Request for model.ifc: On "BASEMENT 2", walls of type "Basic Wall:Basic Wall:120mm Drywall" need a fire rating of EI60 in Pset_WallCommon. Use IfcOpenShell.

First a look at what the model holds.

```python
import ifcopenshell
import ifcopenshell.util.element

model = ifcopenshell.open("model.ifc")
print(model.schema)
storey = next(s for s in model.by_type("IfcBuildingStorey") if s.Name == "BASEMENT 2")
walls = [e for e in ifcopenshell.util.element.get_decomposition(storey) if e.is_a("IfcWall")]
seen = {}
for e in walls:
    element_type = ifcopenshell.util.element.get_type(e)
    key = (element_type.Name if element_type != e and element_type else None, ifcopenshell.util.element.get_pset(e, "Pset_WallCommon", "FireRating"))
    seen[key] = seen.get(key, 0) + 1
for (name, value), count in sorted(seen.items(), key=str):
    print(count, "x", name, "|", value)
```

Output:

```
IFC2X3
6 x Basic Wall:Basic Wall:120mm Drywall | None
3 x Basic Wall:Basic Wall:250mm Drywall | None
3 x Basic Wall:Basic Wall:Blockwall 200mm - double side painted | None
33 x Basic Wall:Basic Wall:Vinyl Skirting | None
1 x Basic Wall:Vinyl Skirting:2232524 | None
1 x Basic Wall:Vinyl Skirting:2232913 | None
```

```python
import ifcopenshell
import ifcopenshell.api.pset
import ifcopenshell.util.element

model = ifcopenshell.open("model.ifc")

storey = next(s for s in model.by_type("IfcBuildingStorey") if s.Name == "BASEMENT 2")
walls = [e for e in ifcopenshell.util.element.get_decomposition(storey) if e.is_a("IfcWall")]

count = 0
for e in walls:
    element_type = ifcopenshell.util.element.get_type(e)
    if element_type in (None, e) or element_type.Name != "Basic Wall:Basic Wall:120mm Drywall":
        continue
    # add_pset returns the element's existing set when there is one.
    pset = ifcopenshell.api.pset.add_pset(model, product=e, name="Pset_WallCommon")
    ifcopenshell.api.pset.edit_pset(model, pset=pset, properties={"FireRating": "EI60"})
    count += 1

print(count, "walls updated")

model.write("model_rev.ifc")
```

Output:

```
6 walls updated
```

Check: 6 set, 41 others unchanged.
